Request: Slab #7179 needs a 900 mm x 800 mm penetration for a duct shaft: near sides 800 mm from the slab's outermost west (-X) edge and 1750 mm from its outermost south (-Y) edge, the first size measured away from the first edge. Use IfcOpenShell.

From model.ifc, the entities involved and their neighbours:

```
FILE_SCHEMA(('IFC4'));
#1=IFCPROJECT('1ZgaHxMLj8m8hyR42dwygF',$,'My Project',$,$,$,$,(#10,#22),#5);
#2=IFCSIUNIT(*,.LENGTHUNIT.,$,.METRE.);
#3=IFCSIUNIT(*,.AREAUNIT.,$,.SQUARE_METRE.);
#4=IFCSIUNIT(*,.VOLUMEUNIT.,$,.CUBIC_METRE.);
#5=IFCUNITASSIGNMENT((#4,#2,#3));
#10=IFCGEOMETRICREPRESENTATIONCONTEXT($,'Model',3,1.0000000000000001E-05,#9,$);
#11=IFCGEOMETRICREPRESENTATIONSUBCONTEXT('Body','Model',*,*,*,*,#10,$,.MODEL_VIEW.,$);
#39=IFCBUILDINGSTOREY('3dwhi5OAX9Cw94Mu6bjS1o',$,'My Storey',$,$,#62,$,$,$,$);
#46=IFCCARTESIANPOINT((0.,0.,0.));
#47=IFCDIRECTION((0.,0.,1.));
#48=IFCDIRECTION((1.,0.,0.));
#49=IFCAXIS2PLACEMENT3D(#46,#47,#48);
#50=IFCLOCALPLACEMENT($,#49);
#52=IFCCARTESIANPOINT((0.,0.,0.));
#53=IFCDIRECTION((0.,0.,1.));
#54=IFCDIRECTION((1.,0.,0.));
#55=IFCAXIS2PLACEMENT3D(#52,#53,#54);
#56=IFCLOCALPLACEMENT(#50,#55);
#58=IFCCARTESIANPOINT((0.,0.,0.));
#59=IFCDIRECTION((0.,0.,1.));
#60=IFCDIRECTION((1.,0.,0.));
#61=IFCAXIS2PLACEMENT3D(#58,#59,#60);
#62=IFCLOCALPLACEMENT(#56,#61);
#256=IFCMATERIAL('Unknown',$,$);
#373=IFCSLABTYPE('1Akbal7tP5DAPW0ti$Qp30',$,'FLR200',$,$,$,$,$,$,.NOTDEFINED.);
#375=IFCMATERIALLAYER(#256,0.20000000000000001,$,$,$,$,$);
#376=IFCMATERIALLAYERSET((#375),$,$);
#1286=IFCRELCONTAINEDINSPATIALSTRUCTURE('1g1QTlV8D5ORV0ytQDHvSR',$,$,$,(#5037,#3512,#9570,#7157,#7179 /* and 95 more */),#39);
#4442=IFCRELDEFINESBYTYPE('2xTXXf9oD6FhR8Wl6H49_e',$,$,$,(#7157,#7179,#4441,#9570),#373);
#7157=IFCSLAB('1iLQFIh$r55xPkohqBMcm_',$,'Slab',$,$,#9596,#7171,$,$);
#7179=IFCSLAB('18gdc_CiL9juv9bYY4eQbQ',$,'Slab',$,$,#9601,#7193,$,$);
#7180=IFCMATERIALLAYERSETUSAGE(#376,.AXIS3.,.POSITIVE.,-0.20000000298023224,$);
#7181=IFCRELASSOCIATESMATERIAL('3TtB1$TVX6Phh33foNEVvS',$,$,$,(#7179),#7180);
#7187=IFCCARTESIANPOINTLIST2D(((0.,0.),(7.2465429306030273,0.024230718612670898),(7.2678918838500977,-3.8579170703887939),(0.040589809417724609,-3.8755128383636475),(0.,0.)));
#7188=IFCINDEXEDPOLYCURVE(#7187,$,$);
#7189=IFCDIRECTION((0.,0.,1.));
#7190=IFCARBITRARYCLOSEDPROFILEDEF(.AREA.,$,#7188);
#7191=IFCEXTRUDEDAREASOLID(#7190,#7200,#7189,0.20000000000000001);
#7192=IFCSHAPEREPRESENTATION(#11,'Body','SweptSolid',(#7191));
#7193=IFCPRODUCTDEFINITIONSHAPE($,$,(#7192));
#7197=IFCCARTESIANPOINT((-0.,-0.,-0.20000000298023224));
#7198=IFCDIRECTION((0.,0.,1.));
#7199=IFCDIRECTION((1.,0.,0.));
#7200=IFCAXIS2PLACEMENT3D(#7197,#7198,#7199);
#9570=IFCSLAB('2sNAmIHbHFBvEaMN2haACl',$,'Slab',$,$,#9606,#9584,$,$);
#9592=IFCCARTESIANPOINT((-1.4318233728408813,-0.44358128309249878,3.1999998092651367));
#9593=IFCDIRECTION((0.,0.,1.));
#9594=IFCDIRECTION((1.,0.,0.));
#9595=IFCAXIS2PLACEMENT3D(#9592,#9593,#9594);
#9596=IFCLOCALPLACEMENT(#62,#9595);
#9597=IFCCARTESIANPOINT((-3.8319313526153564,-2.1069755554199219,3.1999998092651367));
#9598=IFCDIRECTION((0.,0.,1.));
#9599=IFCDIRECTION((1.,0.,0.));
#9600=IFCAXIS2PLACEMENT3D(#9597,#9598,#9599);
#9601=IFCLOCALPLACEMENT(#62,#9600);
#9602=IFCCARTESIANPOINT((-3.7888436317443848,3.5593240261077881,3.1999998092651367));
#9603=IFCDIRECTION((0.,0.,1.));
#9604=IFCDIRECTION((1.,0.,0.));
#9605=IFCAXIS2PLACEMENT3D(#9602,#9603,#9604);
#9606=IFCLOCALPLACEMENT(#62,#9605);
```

```python
import numpy as np
import ifcopenshell
import ifcopenshell.api.feature
import ifcopenshell.api.geometry
import ifcopenshell.api.root
import ifcopenshell.geom
import ifcopenshell.util.placement
import ifcopenshell.util.representation
import ifcopenshell.util.shape
import ifcopenshell.util.unit

model = ifcopenshell.open("model.ifc")
unit_scale = ifcopenshell.util.unit.calculate_unit_scale(model)
settings = ifcopenshell.geom.settings()


def volume(element):
    """Net volume in cubic metres, openings subtracted."""
    shape = ifcopenshell.geom.create_shape(settings, element)
    return ifcopenshell.util.shape.get_volume(shape.geometry)


slab = model.by_id(7179)
before = volume(slab)

# Extent in the slab's own axes, in metres. The edges named are its -X and -Y sides.
slab_shape = ifcopenshell.geom.create_shape(settings, slab)
vertices = ifcopenshell.util.shape.get_vertices(slab_shape.geometry)
x_min, y_min, bottom = vertices.min(axis=0)
top = vertices[:, 2].max()

opening = ifcopenshell.api.root.create_entity(model, ifc_class="IfcOpeningElement", name="Duct shaft opening", predefined_type="OPENING")
context = ifcopenshell.util.representation.get_context(model, "Model", "Body", "MODEL_VIEW")
width, depth = 0.9, 0.8
outline = [(0.0, 0.0), (width, 0.0), (width, depth), (0.0, depth), (0.0, 0.0)]
# Overshoot both faces by 50 mm so the cut is clean.
shape = ifcopenshell.api.geometry.add_slab_representation(
    model, context=context, depth=top - bottom + 0.1, polyline=outline
)
ifcopenshell.api.geometry.assign_representation(model, product=opening, representation=shape)

matrix = ifcopenshell.util.placement.get_local_placement(slab.ObjectPlacement)
matrix[:, 3] = matrix @ np.append(np.array([x_min + 0.8, y_min + 1.75, bottom - 0.05]) / unit_scale, 1.0)
ifcopenshell.api.geometry.edit_object_placement(model, product=opening, matrix=matrix, is_si=False)
ifcopenshell.api.feature.add_feature(model, feature=opening, element=slab)

after = volume(slab)

print(f"slab volume {before:.3f} -> {after:.3f} m3")

model.write("model_rev.ifc")
```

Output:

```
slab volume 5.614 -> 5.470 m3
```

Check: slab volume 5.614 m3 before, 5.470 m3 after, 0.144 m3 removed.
